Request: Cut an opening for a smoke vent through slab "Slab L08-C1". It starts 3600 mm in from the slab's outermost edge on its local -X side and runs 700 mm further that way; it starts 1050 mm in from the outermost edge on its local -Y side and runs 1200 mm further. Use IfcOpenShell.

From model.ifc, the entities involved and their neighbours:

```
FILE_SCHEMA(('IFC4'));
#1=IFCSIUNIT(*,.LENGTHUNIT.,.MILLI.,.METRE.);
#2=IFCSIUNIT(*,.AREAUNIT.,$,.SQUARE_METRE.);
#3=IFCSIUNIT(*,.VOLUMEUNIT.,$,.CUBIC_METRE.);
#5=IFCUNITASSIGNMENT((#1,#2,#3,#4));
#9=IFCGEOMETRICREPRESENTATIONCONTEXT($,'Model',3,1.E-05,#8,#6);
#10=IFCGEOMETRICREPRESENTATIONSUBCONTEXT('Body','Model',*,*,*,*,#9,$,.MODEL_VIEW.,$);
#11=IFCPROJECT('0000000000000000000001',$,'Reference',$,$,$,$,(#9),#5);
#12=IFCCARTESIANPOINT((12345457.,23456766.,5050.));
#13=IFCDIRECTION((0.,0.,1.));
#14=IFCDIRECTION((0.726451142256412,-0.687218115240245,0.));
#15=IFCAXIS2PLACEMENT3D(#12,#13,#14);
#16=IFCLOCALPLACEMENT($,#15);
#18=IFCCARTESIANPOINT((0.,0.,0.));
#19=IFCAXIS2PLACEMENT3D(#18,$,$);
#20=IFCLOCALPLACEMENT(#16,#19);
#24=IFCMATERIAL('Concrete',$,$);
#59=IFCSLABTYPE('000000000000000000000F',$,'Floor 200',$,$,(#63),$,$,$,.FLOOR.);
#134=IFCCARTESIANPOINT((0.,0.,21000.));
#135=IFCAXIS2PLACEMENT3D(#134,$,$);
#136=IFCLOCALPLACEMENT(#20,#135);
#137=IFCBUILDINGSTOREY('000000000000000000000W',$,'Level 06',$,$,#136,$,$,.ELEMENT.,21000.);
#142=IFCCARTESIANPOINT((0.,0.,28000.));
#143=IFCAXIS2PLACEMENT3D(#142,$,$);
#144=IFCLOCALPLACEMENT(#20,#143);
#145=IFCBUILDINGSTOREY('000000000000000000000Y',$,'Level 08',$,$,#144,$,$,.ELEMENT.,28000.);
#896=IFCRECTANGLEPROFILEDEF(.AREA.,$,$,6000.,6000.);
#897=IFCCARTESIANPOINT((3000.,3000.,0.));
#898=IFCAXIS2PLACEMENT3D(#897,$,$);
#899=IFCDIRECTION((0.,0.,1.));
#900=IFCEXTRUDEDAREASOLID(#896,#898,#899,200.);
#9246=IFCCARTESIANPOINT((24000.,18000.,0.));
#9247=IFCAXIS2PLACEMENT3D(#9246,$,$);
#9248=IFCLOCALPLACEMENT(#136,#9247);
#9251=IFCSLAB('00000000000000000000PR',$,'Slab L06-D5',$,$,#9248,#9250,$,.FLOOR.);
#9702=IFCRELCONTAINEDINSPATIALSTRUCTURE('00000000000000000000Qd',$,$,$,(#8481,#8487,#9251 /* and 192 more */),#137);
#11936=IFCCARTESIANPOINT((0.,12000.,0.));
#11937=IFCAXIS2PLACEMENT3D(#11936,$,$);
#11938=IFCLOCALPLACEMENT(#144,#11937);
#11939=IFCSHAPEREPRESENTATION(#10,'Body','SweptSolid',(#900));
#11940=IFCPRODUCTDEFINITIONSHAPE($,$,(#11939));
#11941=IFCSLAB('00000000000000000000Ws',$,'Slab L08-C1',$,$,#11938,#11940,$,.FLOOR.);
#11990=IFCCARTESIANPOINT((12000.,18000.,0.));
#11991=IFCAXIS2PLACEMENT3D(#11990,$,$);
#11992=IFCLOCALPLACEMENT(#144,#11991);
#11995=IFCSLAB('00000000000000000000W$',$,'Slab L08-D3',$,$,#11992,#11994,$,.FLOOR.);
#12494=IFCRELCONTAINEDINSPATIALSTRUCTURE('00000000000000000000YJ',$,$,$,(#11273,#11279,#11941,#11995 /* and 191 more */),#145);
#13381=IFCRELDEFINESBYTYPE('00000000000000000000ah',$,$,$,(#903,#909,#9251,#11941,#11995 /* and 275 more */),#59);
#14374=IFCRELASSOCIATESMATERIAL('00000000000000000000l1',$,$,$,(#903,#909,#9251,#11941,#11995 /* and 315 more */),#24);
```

```python
import numpy as np
import ifcopenshell
import ifcopenshell.api.feature
import ifcopenshell.api.geometry
import ifcopenshell.api.root
import ifcopenshell.geom
import ifcopenshell.util.placement
import ifcopenshell.util.representation
import ifcopenshell.util.shape
import ifcopenshell.util.unit

model = ifcopenshell.open("model.ifc")
unit_scale = ifcopenshell.util.unit.calculate_unit_scale(model)
settings = ifcopenshell.geom.settings()


def volume(element):
    """Net volume in cubic metres, openings subtracted."""
    shape = ifcopenshell.geom.create_shape(settings, element)
    return ifcopenshell.util.shape.get_volume(shape.geometry)


slab = model.by_id(11941)
before = volume(slab)

# Extent in the slab's own axes, in metres. The edges named are its -X and -Y sides.
slab_shape = ifcopenshell.geom.create_shape(settings, slab)
vertices = ifcopenshell.util.shape.get_vertices(slab_shape.geometry)
x_min, y_min, bottom = vertices.min(axis=0)
top = vertices[:, 2].max()

opening = ifcopenshell.api.root.create_entity(model, ifc_class="IfcOpeningElement", name="Smoke vent opening", predefined_type="OPENING")
context = ifcopenshell.util.representation.get_context(model, "Model", "Body", "MODEL_VIEW")
width, depth = 0.7, 1.2
outline = [(0.0, 0.0), (width, 0.0), (width, depth), (0.0, depth), (0.0, 0.0)]
# Overshoot both faces by 50 mm so the cut is clean.
shape = ifcopenshell.api.geometry.add_slab_representation(
    model, context=context, depth=top - bottom + 0.1, polyline=outline
)
ifcopenshell.api.geometry.assign_representation(model, product=opening, representation=shape)

matrix = ifcopenshell.util.placement.get_local_placement(slab.ObjectPlacement)
matrix[:, 3] = matrix @ np.append(np.array([x_min + 3.6, y_min + 1.05, bottom - 0.05]) / unit_scale, 1.0)
ifcopenshell.api.geometry.edit_object_placement(model, product=opening, matrix=matrix, is_si=False)
ifcopenshell.api.feature.add_feature(model, feature=opening, element=slab)

after = volume(slab)

print(f"slab volume {before:.3f} -> {after:.3f} m3")

model.write("model_v2.ifc")
```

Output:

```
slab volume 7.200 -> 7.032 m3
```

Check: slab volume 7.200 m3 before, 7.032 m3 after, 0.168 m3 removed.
